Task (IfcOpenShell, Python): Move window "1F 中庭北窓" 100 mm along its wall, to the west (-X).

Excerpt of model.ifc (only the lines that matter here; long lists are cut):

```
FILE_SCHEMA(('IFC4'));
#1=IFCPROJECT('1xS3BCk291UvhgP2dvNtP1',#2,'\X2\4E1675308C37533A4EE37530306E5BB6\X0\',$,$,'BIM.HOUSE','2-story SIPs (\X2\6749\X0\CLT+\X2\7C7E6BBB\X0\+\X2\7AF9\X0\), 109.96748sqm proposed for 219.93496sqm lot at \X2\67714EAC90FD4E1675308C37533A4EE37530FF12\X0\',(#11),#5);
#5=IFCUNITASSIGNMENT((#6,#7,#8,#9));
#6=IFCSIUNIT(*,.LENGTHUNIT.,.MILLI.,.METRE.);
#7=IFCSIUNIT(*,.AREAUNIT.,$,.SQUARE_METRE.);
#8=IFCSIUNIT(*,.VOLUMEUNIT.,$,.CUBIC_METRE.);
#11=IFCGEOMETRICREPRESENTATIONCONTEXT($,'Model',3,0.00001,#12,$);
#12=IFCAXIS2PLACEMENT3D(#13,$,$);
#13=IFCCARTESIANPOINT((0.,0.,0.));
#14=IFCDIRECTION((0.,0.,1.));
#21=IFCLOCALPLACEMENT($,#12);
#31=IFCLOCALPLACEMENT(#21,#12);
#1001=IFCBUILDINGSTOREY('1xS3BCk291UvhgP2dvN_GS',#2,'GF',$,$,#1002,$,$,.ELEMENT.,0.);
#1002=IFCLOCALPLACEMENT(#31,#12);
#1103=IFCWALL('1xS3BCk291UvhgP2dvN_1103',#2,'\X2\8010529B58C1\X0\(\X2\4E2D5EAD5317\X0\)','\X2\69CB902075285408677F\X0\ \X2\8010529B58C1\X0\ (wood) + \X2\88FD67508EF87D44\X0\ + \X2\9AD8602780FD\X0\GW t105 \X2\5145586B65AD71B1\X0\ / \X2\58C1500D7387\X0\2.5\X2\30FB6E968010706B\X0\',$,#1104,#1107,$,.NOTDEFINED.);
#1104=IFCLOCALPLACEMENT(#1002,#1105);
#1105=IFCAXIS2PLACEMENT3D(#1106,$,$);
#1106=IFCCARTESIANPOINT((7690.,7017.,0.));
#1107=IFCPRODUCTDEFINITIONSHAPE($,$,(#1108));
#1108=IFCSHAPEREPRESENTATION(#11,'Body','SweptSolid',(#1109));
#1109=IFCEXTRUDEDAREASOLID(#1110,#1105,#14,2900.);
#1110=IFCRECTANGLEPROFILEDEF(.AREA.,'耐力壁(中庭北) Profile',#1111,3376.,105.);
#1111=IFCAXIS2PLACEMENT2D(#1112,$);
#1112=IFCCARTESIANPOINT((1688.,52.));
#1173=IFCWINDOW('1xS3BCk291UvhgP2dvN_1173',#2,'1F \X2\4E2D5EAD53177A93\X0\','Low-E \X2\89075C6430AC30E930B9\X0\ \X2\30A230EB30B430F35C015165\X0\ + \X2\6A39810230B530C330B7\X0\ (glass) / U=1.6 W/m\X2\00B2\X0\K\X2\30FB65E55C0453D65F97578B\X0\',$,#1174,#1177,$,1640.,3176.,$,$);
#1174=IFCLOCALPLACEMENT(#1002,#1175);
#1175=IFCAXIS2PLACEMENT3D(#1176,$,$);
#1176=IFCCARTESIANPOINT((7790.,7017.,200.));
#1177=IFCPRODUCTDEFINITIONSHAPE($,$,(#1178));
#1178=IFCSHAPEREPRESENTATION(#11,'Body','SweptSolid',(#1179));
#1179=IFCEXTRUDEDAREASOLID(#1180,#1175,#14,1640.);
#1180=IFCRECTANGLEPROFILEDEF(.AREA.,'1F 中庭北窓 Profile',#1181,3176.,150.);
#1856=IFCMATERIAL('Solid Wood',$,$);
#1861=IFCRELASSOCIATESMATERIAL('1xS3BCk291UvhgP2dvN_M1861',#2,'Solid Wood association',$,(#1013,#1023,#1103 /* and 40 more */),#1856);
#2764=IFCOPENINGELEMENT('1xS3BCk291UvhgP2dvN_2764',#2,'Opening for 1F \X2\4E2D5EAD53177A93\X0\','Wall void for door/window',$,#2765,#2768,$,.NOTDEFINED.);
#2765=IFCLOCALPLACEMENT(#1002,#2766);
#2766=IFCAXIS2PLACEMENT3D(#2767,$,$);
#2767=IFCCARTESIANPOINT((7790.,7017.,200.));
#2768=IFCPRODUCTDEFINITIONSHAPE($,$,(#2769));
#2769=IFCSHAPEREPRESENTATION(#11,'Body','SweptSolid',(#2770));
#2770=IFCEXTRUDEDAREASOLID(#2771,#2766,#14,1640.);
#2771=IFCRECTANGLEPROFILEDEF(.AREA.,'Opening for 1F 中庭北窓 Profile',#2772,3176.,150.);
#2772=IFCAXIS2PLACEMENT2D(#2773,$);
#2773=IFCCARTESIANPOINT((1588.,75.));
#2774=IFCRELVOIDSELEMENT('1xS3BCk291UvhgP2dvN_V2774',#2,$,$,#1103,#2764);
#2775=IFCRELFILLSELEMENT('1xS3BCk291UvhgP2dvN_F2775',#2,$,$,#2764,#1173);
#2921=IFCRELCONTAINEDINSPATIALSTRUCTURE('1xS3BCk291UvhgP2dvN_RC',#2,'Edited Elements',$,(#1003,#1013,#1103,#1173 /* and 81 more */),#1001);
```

```python
import ifcopenshell
import ifcopenshell.api.geometry
import ifcopenshell.util.placement
import ifcopenshell.util.unit

model = ifcopenshell.open("model.ifc")
unit_scale = ifcopenshell.util.unit.calculate_unit_scale(model)

window = model.by_guid("1xS3BCk291UvhgP2dvN_1173")
opening = window.FillsVoids[0].RelatingOpeningElement
wall = opening.VoidsElements[0].RelatingBuildingElement

wall_matrix = ifcopenshell.util.placement.get_local_placement(wall.ObjectPlacement)
shift = wall_matrix[:3, 0] * -0.1 / unit_scale
before = ifcopenshell.util.placement.get_local_placement(window.ObjectPlacement)[:3, 3].copy()

# The window is not placed relative to its opening, so move both.
for product in (opening, window):
    matrix = ifcopenshell.util.placement.get_local_placement(product.ObjectPlacement)
    matrix[:3, 3] += shift
    ifcopenshell.api.geometry.edit_object_placement(model, product=product, matrix=matrix, is_si=False)

after = ifcopenshell.util.placement.get_local_placement(window.ObjectPlacement)[:3, 3]
print("window moved by", (after - before).round(3) + 0.0)

model.write("model_rev.ifc")
```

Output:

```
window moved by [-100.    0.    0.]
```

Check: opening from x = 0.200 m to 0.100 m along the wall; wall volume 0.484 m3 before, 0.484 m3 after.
